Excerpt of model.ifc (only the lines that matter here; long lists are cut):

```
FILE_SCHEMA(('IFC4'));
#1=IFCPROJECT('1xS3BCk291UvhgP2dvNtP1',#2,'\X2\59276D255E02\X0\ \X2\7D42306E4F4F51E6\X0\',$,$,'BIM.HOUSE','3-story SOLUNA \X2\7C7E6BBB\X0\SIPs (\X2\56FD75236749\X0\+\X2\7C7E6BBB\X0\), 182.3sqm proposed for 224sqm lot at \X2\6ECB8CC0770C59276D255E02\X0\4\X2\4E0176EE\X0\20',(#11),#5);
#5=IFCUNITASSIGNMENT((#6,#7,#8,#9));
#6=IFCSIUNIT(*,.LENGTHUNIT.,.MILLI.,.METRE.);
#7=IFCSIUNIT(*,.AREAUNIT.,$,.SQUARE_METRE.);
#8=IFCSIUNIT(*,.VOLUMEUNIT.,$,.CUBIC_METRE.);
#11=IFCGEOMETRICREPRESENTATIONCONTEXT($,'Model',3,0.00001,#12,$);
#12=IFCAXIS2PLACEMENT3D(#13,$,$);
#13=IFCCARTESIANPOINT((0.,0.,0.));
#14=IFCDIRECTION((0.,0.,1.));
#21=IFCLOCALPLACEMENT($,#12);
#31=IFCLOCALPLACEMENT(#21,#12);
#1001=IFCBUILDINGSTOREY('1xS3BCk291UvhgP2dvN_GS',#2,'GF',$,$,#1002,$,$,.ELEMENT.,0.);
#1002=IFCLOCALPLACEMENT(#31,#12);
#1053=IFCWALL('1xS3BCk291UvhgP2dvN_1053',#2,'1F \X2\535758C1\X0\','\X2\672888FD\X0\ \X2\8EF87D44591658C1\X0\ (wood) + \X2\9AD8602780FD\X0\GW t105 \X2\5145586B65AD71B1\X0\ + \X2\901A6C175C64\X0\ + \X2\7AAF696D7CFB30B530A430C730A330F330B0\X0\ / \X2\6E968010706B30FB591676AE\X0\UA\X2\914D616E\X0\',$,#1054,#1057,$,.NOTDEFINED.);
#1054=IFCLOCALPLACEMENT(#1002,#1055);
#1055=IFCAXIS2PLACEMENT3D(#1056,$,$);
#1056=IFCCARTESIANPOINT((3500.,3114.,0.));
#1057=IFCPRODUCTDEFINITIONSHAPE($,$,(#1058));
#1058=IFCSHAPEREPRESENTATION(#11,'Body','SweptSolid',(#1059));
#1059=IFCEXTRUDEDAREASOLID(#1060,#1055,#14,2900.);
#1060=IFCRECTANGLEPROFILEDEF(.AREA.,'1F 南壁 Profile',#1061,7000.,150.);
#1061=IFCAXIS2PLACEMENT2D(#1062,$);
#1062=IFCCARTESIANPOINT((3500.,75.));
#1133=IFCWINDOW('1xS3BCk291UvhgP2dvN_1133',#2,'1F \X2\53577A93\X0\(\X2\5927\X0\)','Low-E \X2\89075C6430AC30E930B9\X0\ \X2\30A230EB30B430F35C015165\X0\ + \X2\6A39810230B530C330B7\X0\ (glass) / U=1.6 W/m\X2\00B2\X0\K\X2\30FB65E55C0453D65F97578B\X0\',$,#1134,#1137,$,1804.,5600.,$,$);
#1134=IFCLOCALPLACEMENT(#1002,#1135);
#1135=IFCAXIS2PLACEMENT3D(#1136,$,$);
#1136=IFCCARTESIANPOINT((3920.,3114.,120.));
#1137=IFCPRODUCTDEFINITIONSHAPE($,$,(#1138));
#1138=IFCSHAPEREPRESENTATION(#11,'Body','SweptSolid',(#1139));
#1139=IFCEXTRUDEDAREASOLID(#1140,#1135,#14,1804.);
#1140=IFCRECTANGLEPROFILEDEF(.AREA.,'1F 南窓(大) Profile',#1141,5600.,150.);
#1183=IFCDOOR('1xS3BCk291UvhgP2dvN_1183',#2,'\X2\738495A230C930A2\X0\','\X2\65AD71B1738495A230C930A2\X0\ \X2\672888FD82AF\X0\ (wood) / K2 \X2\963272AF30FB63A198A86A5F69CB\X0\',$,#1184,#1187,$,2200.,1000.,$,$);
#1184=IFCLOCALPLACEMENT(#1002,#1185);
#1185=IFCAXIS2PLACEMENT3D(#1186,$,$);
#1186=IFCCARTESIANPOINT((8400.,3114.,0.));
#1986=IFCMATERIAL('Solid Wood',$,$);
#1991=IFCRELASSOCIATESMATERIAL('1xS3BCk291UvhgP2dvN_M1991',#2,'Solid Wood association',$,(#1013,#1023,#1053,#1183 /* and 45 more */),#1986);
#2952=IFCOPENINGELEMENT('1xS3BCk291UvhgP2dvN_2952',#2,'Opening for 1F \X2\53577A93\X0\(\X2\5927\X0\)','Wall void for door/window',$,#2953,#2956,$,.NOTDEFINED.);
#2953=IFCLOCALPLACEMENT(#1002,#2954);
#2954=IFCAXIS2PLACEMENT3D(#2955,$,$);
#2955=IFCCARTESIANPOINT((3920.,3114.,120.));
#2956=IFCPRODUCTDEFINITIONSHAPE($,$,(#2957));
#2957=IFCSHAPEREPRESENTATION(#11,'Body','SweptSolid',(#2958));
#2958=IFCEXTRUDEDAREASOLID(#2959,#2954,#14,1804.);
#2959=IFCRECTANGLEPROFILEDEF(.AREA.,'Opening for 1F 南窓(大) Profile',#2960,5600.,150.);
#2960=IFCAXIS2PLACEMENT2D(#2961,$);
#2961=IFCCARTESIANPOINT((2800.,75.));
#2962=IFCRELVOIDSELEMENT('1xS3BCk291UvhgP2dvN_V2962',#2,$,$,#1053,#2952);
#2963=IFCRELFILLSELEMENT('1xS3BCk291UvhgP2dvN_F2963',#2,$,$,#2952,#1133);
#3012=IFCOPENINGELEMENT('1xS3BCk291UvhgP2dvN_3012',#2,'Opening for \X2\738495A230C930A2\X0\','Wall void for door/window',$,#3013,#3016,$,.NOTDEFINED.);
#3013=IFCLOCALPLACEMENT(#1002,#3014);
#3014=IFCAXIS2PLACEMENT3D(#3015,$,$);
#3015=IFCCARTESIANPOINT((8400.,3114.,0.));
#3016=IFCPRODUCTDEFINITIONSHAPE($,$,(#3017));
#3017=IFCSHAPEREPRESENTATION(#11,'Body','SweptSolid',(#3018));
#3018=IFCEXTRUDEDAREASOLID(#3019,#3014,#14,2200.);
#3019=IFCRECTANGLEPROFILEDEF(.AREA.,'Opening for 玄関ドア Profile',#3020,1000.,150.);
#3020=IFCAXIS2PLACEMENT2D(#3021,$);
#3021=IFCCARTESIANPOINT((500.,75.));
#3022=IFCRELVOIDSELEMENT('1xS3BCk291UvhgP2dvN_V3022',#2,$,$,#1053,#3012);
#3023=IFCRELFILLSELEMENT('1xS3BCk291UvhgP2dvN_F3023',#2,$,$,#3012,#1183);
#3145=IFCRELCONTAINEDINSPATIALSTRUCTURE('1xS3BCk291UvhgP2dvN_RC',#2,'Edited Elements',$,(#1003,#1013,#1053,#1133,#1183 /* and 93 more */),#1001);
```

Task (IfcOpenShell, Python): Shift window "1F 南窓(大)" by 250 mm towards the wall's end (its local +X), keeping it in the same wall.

```python
import ifcopenshell
import ifcopenshell.api.geometry
import ifcopenshell.util.placement

model = ifcopenshell.open("model.ifc")

window = model.by_guid("1xS3BCk291UvhgP2dvN_1133")
opening = window.FillsVoids[0].RelatingOpeningElement
wall = opening.VoidsElements[0].RelatingBuildingElement

wall_matrix = ifcopenshell.util.placement.get_local_placement(wall.ObjectPlacement)
shift = wall_matrix[:3, 0] * 250.0
before = ifcopenshell.util.placement.get_local_placement(window.ObjectPlacement)[:3, 3].copy()

# The window is not placed relative to its opening, so move both.
for product in (opening, window):
    matrix = ifcopenshell.util.placement.get_local_placement(product.ObjectPlacement)
    matrix[:3, 3] += shift
    ifcopenshell.api.geometry.edit_object_placement(model, product=product, matrix=matrix, is_si=False)

after = ifcopenshell.util.placement.get_local_placement(window.ObjectPlacement)[:3, 3]
print("window moved by", (after - before).round(3) + 0.0)

model.write("model-out.ifc")
```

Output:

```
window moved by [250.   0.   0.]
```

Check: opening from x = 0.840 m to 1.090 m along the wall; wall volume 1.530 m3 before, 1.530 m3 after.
